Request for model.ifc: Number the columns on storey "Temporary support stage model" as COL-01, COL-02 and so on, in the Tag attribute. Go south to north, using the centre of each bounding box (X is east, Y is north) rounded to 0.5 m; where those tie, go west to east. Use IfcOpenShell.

First a look at what the model holds.

```python
import ifcopenshell
import ifcopenshell.util.element
import ifcopenshell.util.placement

model = ifcopenshell.open("model.ifc")
print(model.schema)
storey = next(s for s in model.by_type("IfcBuildingStorey") if s.Name == "Temporary support stage model")
columns = [e for e in ifcopenshell.util.element.get_decomposition(storey) if e.is_a("IfcColumn")]
for e in sorted(columns, key=lambda e: e.id()):
    origin = ifcopenshell.util.placement.get_local_placement(e.ObjectPlacement)[:3, 3]
    print(e.id(), e.Tag, e.Name, origin.round(2) + 0.0, sep=" | ")
```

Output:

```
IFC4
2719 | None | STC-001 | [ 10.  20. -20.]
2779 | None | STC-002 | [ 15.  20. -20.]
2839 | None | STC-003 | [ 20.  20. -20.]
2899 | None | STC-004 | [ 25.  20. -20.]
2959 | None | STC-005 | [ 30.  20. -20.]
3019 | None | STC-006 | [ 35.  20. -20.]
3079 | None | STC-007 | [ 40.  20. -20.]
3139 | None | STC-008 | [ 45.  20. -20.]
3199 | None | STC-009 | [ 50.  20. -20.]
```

```python
import ifcopenshell
import ifcopenshell.geom
import ifcopenshell.util.element
import ifcopenshell.util.shape

model = ifcopenshell.open("model.ifc")
settings = ifcopenshell.geom.settings()
settings.set("use-world-coords", True)


def centre(element):
    shape = ifcopenshell.geom.create_shape(settings, element)
    return ifcopenshell.util.shape.get_bbox_centroid(shape.geometry)


storey = next(s for s in model.by_type("IfcBuildingStorey") if s.Name == "Temporary support stage model")
columns = [e for e in ifcopenshell.util.element.get_decomposition(storey) if e.is_a("IfcColumn")]

# Insertion points can sit at a corner or the storey origin, so sort by the geometry (in metres).
centres = {e: centre(e) for e in columns}
columns.sort(key=lambda e: (round(centres[e][1] / 0.5), centres[e][0]))

for i, e in enumerate(columns, start=1):
    number = f"COL-{i:02d}"
    e.Tag = number
    print(e.id(), number)

model.write("model_updated.ifc")
```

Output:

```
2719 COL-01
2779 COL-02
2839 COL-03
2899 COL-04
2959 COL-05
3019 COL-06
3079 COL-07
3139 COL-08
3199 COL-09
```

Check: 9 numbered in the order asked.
